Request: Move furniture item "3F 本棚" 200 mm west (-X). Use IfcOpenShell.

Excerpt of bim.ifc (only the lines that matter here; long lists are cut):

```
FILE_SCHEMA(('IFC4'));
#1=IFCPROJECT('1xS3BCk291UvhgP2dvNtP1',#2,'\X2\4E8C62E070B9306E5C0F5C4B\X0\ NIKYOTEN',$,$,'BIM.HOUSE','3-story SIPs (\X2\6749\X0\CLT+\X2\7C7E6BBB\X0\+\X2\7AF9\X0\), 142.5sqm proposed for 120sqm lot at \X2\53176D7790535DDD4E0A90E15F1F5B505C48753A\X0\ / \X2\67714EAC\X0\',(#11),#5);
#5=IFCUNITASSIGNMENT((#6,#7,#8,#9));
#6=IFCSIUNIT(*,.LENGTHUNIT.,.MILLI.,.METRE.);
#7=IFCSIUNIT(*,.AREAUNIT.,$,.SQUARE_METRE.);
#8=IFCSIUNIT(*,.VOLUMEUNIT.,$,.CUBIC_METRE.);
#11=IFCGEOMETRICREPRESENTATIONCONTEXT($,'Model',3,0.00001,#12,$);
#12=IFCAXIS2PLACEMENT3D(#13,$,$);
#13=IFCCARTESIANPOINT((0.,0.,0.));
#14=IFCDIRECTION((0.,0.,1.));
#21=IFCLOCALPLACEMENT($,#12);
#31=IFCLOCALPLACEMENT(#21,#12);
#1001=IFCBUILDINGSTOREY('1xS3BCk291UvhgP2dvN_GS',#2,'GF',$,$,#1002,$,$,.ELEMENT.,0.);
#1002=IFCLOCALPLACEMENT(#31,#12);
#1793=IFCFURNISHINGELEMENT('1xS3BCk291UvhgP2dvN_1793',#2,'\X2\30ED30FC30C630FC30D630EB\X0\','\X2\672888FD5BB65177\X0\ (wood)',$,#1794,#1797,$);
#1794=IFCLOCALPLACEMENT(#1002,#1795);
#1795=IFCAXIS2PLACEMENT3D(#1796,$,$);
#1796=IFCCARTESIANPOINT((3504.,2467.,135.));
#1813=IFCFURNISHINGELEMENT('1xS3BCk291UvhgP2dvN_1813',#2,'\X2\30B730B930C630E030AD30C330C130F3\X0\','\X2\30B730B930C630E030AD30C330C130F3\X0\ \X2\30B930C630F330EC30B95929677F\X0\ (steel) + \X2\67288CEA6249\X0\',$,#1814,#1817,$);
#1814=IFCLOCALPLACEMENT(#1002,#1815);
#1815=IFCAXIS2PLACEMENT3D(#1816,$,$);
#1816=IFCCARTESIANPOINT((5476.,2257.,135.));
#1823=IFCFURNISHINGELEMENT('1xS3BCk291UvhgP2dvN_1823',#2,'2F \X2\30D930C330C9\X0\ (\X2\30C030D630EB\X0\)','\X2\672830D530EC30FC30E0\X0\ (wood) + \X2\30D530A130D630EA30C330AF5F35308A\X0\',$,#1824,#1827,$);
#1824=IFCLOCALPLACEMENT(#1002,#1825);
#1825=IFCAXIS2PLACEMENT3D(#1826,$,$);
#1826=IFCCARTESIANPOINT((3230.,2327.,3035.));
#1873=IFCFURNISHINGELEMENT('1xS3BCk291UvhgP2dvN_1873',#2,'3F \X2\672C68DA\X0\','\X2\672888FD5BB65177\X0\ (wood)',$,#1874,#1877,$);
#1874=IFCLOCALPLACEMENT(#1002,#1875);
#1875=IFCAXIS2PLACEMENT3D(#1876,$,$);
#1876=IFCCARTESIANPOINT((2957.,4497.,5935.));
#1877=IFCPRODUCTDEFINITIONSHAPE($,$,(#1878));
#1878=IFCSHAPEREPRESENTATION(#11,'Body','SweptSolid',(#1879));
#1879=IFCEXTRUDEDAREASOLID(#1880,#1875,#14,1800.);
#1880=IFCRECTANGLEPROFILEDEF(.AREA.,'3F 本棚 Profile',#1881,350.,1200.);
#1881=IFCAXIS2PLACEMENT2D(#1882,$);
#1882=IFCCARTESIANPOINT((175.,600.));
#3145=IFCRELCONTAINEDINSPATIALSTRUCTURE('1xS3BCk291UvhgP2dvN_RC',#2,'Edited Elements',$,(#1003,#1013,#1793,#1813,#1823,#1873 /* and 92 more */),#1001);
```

```python
import ifcopenshell
import ifcopenshell.api.geometry
import ifcopenshell.util.placement

model = ifcopenshell.open("bim.ifc")

item = model.by_guid("1xS3BCk291UvhgP2dvN_1873")
matrix = ifcopenshell.util.placement.get_local_placement(item.ObjectPlacement)
matrix[0, 3] -= 200.0
ifcopenshell.api.geometry.edit_object_placement(model, product=item, matrix=matrix, is_si=False)

print(ifcopenshell.util.placement.get_local_placement(item.ObjectPlacement).round(3) + 0.0)

model.write("bim_updated.ifc")
```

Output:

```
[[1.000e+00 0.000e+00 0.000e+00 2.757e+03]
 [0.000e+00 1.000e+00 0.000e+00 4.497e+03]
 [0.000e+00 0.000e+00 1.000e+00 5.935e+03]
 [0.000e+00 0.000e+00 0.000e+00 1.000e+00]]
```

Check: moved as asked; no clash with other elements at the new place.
